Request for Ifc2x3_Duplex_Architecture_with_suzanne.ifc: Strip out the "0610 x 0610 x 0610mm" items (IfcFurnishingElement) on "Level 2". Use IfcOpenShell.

First a look at what the model holds.

```python
import ifcopenshell
import ifcopenshell.util.element

model = ifcopenshell.open("Ifc2x3_Duplex_Architecture_with_suzanne.ifc")
print(model.schema)
storey = next(s for s in model.by_type("IfcBuildingStorey") if s.Name == "Level 2")
furniture = [e for e in ifcopenshell.util.element.get_decomposition(storey) if e.is_a("IfcFurnishingElement")]
seen = {}
for e in furniture:
    element_type = ifcopenshell.util.element.get_type(e)
    name = element_type.Name if element_type not in (None, e) else None
    seen[name] = seen.get(name, 0) + 1
for name, count in sorted(seen.items(), key=str):
    print(count, "x", name)
```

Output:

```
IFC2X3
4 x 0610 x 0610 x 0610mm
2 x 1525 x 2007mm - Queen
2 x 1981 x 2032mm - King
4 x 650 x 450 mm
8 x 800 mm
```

```python
import ifcopenshell
import ifcopenshell.api.root
import ifcopenshell.util.element

model = ifcopenshell.open("Ifc2x3_Duplex_Architecture_with_suzanne.ifc")

storey = next(s for s in model.by_type("IfcBuildingStorey") if s.Name == "Level 2")
furniture = [e for e in ifcopenshell.util.element.get_decomposition(storey) if e.is_a("IfcFurnishingElement")]
targets = [e for e in furniture if (t := ifcopenshell.util.element.get_type(e)) not in (None, e) and t.Name == "0610 x 0610 x 0610mm"]

for e in targets:
    ifcopenshell.api.root.remove_product(model, product=e)
print(len(targets), "removed")

model.write("Ifc2x3_Duplex_Architecture_with_suzanne_v2.ifc")
```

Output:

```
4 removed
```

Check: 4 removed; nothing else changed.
